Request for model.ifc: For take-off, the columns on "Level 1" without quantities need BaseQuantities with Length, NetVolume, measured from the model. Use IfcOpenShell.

First a look at what the model holds.

```python
import ifcopenshell
import ifcopenshell.util.element
import ifcopenshell.util.unit

model = ifcopenshell.open("model.ifc")
print(model.schema)
for unit_type in ("LENGTHUNIT", "AREAUNIT", "VOLUMEUNIT"):
    print(unit_type, ifcopenshell.util.unit.calculate_unit_scale(model, unit_type))
storey = next(s for s in model.by_type("IfcBuildingStorey") if s.Name == "Level 1")
columns = [e for e in ifcopenshell.util.element.get_decomposition(storey) if e.is_a("IfcColumn")]
for e in sorted(columns, key=lambda e: e.id()):
    print(e.id(), e.is_a(), e.Name, list(ifcopenshell.util.element.get_psets(e, qtos_only=True)), sep=" | ")
```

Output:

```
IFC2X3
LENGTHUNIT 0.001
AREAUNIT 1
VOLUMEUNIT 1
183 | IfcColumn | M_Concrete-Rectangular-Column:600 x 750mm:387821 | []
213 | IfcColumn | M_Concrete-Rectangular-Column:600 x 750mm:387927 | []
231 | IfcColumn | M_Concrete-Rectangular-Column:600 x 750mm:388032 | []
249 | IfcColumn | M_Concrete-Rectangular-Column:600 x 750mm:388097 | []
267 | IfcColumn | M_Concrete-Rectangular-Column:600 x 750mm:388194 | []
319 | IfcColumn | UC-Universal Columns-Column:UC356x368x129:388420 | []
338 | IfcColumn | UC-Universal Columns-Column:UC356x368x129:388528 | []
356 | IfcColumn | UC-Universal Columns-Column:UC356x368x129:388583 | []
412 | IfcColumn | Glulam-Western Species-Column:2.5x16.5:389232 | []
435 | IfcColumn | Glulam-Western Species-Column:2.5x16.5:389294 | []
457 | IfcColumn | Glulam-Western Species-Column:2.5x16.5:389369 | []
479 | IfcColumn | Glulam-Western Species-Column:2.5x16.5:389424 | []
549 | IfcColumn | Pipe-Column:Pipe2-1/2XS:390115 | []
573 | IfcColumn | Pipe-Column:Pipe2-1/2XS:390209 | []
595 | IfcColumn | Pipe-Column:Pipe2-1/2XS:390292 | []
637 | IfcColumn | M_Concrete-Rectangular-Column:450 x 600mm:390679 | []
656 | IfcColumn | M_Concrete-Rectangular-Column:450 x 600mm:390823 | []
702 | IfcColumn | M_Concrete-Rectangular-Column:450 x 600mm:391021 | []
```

```python
import ifcopenshell
import ifcopenshell.api.pset
import ifcopenshell.geom
import ifcopenshell.util.element
import ifcopenshell.util.shape
import ifcopenshell.util.unit

model = ifcopenshell.open("model.ifc")
unit_scale = ifcopenshell.util.unit.calculate_unit_scale(model)
volume_scale = ifcopenshell.util.unit.calculate_unit_scale(model, "VOLUMEUNIT")
settings = ifcopenshell.geom.settings()

storey = next(s for s in model.by_type("IfcBuildingStorey") if s.Name == "Level 1")
columns = [e for e in ifcopenshell.util.element.get_decomposition(storey) if e.is_a("IfcColumn")]

for e in sorted(columns, key=lambda e: e.id()):
    if ifcopenshell.util.element.get_psets(e, qtos_only=True, should_inherit=False):
        continue
    # Geometry comes back in metres, in the element's own axes.
    shape = ifcopenshell.geom.create_shape(settings, e)
    values = {
        "Length": ifcopenshell.util.shape.get_z(shape.geometry) / unit_scale,
        "NetVolume": ifcopenshell.util.shape.get_volume(shape.geometry) / volume_scale,
    }
    qto = ifcopenshell.api.pset.add_qto(model, product=e, name="BaseQuantities")
    ifcopenshell.api.pset.edit_qto(model, qto=qto, properties=values)
    print(e.id(), {k: round(v, 3) for k, v in values.items()})

model.write("model_edited.ifc")
```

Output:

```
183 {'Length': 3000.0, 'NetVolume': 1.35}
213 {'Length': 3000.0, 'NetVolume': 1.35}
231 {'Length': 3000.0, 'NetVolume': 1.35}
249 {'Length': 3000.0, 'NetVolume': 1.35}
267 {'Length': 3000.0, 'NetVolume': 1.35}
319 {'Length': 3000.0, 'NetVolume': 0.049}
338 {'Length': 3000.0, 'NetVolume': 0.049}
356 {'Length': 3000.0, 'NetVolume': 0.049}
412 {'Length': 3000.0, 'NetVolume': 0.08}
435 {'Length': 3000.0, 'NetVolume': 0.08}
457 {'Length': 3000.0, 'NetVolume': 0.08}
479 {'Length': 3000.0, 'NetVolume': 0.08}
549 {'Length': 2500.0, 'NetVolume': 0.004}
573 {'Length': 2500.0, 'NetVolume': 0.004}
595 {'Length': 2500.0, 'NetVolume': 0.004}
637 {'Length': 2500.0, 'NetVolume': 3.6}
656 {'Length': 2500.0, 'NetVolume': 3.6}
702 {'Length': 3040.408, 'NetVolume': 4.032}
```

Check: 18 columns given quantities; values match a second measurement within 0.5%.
